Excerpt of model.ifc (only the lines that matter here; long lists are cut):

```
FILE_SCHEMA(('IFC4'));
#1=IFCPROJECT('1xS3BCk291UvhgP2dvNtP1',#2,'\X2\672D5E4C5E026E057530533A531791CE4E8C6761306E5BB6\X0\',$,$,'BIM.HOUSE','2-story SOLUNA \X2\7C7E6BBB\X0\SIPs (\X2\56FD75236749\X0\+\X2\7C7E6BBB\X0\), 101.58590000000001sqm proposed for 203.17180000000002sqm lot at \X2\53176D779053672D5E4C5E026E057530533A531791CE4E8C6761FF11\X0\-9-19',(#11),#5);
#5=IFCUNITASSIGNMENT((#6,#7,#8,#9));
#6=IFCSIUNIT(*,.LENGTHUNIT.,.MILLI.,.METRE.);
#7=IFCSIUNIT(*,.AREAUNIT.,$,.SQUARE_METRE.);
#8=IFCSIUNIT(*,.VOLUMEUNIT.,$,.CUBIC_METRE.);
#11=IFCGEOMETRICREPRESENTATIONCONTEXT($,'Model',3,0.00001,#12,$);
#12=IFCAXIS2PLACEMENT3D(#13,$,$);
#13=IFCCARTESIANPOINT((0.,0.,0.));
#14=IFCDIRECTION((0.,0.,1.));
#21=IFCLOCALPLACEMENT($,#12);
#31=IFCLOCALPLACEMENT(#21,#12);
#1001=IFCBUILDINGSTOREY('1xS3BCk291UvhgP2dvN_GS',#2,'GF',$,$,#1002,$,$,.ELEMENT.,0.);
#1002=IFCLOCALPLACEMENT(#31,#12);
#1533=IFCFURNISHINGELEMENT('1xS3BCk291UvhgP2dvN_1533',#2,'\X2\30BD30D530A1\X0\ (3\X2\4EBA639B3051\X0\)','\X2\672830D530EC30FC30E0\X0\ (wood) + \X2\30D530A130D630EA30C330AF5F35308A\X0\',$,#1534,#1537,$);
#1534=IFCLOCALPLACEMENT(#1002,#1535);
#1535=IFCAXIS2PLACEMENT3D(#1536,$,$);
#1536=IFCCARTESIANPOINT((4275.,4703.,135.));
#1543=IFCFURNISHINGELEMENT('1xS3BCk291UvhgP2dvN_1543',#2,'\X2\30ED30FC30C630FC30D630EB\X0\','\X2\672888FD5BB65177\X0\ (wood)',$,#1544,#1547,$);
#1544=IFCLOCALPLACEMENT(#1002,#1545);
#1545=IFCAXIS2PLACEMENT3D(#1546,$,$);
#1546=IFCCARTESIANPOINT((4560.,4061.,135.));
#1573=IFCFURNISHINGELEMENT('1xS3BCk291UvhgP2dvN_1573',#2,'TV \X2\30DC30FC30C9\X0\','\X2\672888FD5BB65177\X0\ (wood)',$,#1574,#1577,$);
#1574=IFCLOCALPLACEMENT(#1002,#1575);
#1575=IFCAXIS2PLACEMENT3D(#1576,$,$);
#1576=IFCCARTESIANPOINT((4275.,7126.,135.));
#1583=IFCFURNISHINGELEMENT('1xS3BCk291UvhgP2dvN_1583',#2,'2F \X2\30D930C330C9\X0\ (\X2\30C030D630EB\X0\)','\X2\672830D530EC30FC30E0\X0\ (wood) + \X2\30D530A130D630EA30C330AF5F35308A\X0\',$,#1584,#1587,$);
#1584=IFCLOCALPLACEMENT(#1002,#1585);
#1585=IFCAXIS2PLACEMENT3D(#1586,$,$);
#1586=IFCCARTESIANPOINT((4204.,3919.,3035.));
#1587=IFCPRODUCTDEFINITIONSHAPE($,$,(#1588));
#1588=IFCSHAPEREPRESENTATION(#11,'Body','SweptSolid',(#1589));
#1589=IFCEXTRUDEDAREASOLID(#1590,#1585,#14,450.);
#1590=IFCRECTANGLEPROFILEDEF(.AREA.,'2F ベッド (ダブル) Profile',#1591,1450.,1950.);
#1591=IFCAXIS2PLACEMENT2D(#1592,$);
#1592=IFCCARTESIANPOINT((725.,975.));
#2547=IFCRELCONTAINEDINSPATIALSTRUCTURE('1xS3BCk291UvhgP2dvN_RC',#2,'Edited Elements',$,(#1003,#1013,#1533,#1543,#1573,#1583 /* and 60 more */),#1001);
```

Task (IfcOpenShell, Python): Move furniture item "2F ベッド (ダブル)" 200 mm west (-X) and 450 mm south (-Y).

```python
import ifcopenshell
import ifcopenshell.api.geometry
import ifcopenshell.util.placement
import ifcopenshell.util.unit

model = ifcopenshell.open("model.ifc")
unit_scale = ifcopenshell.util.unit.calculate_unit_scale(model)

item = model.by_id(1583)
matrix = ifcopenshell.util.placement.get_local_placement(item.ObjectPlacement)
matrix[0, 3] -= 0.2 / unit_scale
matrix[1, 3] -= 0.45 / unit_scale
ifcopenshell.api.geometry.edit_object_placement(model, product=item, matrix=matrix, is_si=False)

print(ifcopenshell.util.placement.get_local_placement(item.ObjectPlacement).round(3) + 0.0)

model.write("model_rev.ifc")
```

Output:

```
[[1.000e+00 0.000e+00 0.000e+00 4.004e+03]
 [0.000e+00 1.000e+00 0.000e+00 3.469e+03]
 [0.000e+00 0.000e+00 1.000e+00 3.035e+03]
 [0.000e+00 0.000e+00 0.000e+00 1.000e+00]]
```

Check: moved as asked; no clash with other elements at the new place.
